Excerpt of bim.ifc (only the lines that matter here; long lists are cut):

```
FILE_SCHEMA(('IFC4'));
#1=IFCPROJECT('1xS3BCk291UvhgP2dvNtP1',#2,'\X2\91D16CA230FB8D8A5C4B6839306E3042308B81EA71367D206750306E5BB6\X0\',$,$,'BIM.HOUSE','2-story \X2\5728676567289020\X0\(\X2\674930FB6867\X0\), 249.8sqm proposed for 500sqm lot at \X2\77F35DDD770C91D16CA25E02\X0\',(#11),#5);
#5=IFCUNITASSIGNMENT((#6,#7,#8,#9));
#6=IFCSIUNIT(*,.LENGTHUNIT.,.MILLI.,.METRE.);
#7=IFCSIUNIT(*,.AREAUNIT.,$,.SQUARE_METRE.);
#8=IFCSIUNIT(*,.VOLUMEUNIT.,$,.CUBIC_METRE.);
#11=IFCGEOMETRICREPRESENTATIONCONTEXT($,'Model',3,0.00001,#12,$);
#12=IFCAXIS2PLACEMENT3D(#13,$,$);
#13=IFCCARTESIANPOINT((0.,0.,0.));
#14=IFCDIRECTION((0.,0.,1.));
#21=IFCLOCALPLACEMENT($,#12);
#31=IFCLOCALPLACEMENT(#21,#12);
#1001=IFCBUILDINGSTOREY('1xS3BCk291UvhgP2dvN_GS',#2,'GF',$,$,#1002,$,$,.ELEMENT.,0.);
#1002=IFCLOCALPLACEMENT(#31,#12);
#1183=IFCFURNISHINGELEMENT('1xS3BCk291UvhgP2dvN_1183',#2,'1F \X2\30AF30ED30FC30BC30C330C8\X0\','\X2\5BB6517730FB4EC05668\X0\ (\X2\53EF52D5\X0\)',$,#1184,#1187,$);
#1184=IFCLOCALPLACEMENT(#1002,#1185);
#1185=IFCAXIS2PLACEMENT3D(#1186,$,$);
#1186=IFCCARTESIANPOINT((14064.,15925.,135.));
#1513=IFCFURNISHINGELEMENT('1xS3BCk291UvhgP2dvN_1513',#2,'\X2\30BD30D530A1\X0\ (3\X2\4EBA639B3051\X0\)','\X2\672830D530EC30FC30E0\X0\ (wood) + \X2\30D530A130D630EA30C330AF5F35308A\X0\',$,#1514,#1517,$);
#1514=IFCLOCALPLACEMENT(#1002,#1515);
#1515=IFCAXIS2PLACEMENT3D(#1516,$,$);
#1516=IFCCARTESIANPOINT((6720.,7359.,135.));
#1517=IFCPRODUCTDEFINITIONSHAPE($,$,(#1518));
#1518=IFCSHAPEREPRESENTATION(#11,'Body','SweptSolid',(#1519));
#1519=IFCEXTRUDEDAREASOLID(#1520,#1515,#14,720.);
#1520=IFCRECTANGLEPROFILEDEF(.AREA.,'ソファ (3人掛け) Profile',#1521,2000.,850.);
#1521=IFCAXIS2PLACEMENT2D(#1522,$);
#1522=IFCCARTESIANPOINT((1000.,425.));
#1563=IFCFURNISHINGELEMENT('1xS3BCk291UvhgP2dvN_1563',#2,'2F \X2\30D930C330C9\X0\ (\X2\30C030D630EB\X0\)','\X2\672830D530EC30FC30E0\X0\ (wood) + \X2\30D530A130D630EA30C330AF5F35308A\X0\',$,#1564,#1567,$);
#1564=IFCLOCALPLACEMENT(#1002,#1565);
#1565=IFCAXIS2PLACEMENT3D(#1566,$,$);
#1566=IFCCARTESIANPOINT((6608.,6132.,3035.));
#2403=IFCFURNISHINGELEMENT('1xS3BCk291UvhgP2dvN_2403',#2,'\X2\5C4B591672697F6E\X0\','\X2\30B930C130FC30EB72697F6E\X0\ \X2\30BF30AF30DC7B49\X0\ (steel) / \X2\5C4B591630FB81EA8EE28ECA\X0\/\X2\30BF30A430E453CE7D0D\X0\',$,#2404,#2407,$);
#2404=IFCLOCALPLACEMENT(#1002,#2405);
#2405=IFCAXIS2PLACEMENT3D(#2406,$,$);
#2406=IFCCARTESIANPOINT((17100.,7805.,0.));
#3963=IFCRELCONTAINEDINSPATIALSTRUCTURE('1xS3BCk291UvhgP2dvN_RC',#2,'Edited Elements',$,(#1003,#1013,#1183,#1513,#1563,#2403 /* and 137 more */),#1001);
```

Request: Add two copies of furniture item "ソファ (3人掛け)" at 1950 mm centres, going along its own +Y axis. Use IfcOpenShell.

```python
import ifcopenshell
import ifcopenshell.api.geometry
import ifcopenshell.api.root
import ifcopenshell.util.element
import ifcopenshell.util.placement

model = ifcopenshell.open("bim.ifc")


def reuse_history(source, copy):
    """copy_class also copies each property set's owner history, people and application; keep the originals."""
    for rel in copy.IsDefinedBy:
        if rel.is_a("IfcRelDefinesByProperties") and (history := rel.RelatingPropertyDefinition.OwnerHistory):
            rel.RelatingPropertyDefinition.OwnerHistory = source.OwnerHistory
            ifcopenshell.util.element.remove_deep2(model, history)


source = model.by_guid("1xS3BCk291UvhgP2dvN_1513")
base = ifcopenshell.util.placement.get_local_placement(source.ObjectPlacement)
step = base[:3, 1] * 1950.0

for i in range(1, 3):
    copy = ifcopenshell.api.root.copy_class(model, product=source)
    copy.Representation = ifcopenshell.util.element.copy_deep(
        model, source.Representation, exclude=["IfcGeometricRepresentationContext", "IfcRepresentationMap"]
    )
    reuse_history(source, copy)
    matrix = base.copy()
    matrix[:3, 3] += i * step
    print("added at", matrix[:3, 3].round(3) + 0.0)
    ifcopenshell.api.geometry.edit_object_placement(model, product=copy, matrix=matrix, is_si=False)

model.write("bim_rev.ifc")
```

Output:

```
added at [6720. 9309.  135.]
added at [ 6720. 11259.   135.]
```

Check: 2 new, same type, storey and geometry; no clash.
